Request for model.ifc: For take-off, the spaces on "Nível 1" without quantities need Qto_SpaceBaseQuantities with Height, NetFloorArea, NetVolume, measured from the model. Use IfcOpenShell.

First a look at what the model holds.

```python
import ifcopenshell
import ifcopenshell.util.element
import ifcopenshell.util.unit

model = ifcopenshell.open("model.ifc")
print(model.schema)
for unit_type in ("LENGTHUNIT", "AREAUNIT", "VOLUMEUNIT"):
    print(unit_type, ifcopenshell.util.unit.calculate_unit_scale(model, unit_type))
storey = next(s for s in model.by_type("IfcBuildingStorey") if s.Name == "Nível 1")
spaces = [e for e in ifcopenshell.util.element.get_decomposition(storey) if e.is_a("IfcSpace")]
for e in sorted(spaces, key=lambda e: e.id()):
    print(e.id(), e.is_a(), e.Name, list(ifcopenshell.util.element.get_psets(e, qtos_only=True)), sep=" | ")
```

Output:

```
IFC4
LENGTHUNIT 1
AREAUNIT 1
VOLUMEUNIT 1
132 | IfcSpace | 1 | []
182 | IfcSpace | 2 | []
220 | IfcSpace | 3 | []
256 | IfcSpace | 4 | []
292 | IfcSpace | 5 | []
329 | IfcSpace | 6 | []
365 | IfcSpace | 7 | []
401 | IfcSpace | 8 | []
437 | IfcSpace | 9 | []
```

```python
import ifcopenshell
import ifcopenshell.api.pset
import ifcopenshell.geom
import ifcopenshell.util.element
import ifcopenshell.util.shape
import ifcopenshell.util.unit

model = ifcopenshell.open("model.ifc")
unit_scale = ifcopenshell.util.unit.calculate_unit_scale(model)
area_scale = ifcopenshell.util.unit.calculate_unit_scale(model, "AREAUNIT")
volume_scale = ifcopenshell.util.unit.calculate_unit_scale(model, "VOLUMEUNIT")
settings = ifcopenshell.geom.settings()

storey = next(s for s in model.by_type("IfcBuildingStorey") if s.Name == "Nível 1")
spaces = [e for e in ifcopenshell.util.element.get_decomposition(storey) if e.is_a("IfcSpace")]

for e in sorted(spaces, key=lambda e: e.id()):
    if ifcopenshell.util.element.get_psets(e, qtos_only=True, should_inherit=False):
        continue
    # Geometry comes back in metres, in the element's own axes.
    shape = ifcopenshell.geom.create_shape(settings, e)
    values = {
        "Height": ifcopenshell.util.shape.get_z(shape.geometry) / unit_scale,
        "NetFloorArea": ifcopenshell.util.shape.get_footprint_area(shape.geometry) / area_scale,
        "NetVolume": ifcopenshell.util.shape.get_volume(shape.geometry) / volume_scale,
    }
    qto = ifcopenshell.api.pset.add_qto(model, product=e, name="Qto_SpaceBaseQuantities")
    ifcopenshell.api.pset.edit_qto(model, qto=qto, properties=values)
    print(e.id(), {k: round(v, 3) for k, v in values.items()})

model.write("model_edited.ifc")
```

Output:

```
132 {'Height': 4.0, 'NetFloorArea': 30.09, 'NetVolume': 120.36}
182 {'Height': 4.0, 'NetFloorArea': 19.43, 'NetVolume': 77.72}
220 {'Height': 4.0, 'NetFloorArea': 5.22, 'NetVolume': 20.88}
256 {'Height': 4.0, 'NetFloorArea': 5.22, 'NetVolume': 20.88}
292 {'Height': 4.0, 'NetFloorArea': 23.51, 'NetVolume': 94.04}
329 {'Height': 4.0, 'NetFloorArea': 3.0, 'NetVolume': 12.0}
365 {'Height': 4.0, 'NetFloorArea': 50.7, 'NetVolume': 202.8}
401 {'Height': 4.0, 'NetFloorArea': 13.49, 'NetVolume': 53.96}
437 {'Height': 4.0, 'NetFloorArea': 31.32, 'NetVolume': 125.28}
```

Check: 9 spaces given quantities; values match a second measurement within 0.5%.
